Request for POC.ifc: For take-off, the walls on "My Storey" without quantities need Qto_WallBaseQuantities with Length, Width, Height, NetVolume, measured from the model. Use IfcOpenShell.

First a look at what the model holds.

```python
import ifcopenshell
import ifcopenshell.util.element
import ifcopenshell.util.unit

model = ifcopenshell.open("POC.ifc")
print(model.schema)
for unit_type in ("LENGTHUNIT", "AREAUNIT", "VOLUMEUNIT"):
    print(unit_type, ifcopenshell.util.unit.calculate_unit_scale(model, unit_type))
storey = next(s for s in model.by_type("IfcBuildingStorey") if s.Name == "My Storey")
walls = [e for e in ifcopenshell.util.element.get_decomposition(storey) if e.is_a("IfcWall")]
for e in sorted(walls, key=lambda e: e.id()):
    print(e.id(), e.is_a(), e.Name, list(ifcopenshell.util.element.get_psets(e, qtos_only=True)), sep=" | ")
```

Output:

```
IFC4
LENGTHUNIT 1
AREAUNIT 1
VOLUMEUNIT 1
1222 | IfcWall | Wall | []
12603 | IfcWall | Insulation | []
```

```python
import ifcopenshell
import ifcopenshell.api.pset
import ifcopenshell.geom
import ifcopenshell.util.element
import ifcopenshell.util.shape
import ifcopenshell.util.unit

model = ifcopenshell.open("POC.ifc")
unit_scale = ifcopenshell.util.unit.calculate_unit_scale(model)
volume_scale = ifcopenshell.util.unit.calculate_unit_scale(model, "VOLUMEUNIT")
settings = ifcopenshell.geom.settings()

storey = next(s for s in model.by_type("IfcBuildingStorey") if s.Name == "My Storey")
walls = [e for e in ifcopenshell.util.element.get_decomposition(storey) if e.is_a("IfcWall")]

for e in sorted(walls, key=lambda e: e.id()):
    if ifcopenshell.util.element.get_psets(e, qtos_only=True, should_inherit=False):
        continue
    # Geometry comes back in metres, in the element's own axes.
    shape = ifcopenshell.geom.create_shape(settings, e)
    values = {
        "Length": ifcopenshell.util.shape.get_x(shape.geometry) / unit_scale,
        "Width": ifcopenshell.util.shape.get_y(shape.geometry) / unit_scale,
        "Height": ifcopenshell.util.shape.get_z(shape.geometry) / unit_scale,
        "NetVolume": ifcopenshell.util.shape.get_volume(shape.geometry) / volume_scale,
    }
    qto = ifcopenshell.api.pset.add_qto(model, product=e, name="Qto_WallBaseQuantities")
    ifcopenshell.api.pset.edit_qto(model, qto=qto, properties=values)
    print(e.id(), {k: round(v, 3) for k, v in values.items()})

model.write("POC_updated.ifc")
```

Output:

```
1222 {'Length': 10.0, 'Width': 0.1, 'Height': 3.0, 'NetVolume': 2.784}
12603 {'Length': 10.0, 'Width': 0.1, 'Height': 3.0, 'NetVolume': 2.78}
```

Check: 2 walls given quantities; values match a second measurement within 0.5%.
